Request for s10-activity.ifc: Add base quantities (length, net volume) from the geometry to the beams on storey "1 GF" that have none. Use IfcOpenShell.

First a look at what the model holds.

```python
import ifcopenshell
import ifcopenshell.util.element
import ifcopenshell.util.unit

model = ifcopenshell.open("s10-activity.ifc")
print(model.schema)
for unit_type in ("LENGTHUNIT", "AREAUNIT", "VOLUMEUNIT"):
    print(unit_type, ifcopenshell.util.unit.calculate_unit_scale(model, unit_type))
storey = next(s for s in model.by_type("IfcBuildingStorey") if s.Name == "1 GF")
beams = [e for e in ifcopenshell.util.element.get_decomposition(storey) if e.is_a("IfcBeam")]
for e in sorted(beams, key=lambda e: e.id()):
    print(e.id(), e.is_a(), e.Name, list(ifcopenshell.util.element.get_psets(e, qtos_only=True)), sep=" | ")
```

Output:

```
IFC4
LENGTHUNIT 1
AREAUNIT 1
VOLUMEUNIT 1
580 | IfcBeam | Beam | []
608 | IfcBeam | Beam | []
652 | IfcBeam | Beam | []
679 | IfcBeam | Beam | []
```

```python
import ifcopenshell
import ifcopenshell.api.pset
import ifcopenshell.geom
import ifcopenshell.util.element
import ifcopenshell.util.shape
import ifcopenshell.util.unit

model = ifcopenshell.open("s10-activity.ifc")
unit_scale = ifcopenshell.util.unit.calculate_unit_scale(model)
volume_scale = ifcopenshell.util.unit.calculate_unit_scale(model, "VOLUMEUNIT")
settings = ifcopenshell.geom.settings()

storey = next(s for s in model.by_type("IfcBuildingStorey") if s.Name == "1 GF")
beams = [e for e in ifcopenshell.util.element.get_decomposition(storey) if e.is_a("IfcBeam")]

for e in sorted(beams, key=lambda e: e.id()):
    if ifcopenshell.util.element.get_psets(e, qtos_only=True, should_inherit=False):
        continue
    # Geometry comes back in metres, in the element's own axes.
    shape = ifcopenshell.geom.create_shape(settings, e)
    values = {
        "Length": ifcopenshell.util.shape.get_max_xyz(shape.geometry) / unit_scale,
        "NetVolume": ifcopenshell.util.shape.get_volume(shape.geometry) / volume_scale,
    }
    qto = ifcopenshell.api.pset.add_qto(model, product=e, name="Qto_BeamBaseQuantities")
    ifcopenshell.api.pset.edit_qto(model, qto=qto, properties=values)
    print(e.id(), {k: round(v, 3) for k, v in values.items()})

model.write("s10-activity_rev.ifc")
```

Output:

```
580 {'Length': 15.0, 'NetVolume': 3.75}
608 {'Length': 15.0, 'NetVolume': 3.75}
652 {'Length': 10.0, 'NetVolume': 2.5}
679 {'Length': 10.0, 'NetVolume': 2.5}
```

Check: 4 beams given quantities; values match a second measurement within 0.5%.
